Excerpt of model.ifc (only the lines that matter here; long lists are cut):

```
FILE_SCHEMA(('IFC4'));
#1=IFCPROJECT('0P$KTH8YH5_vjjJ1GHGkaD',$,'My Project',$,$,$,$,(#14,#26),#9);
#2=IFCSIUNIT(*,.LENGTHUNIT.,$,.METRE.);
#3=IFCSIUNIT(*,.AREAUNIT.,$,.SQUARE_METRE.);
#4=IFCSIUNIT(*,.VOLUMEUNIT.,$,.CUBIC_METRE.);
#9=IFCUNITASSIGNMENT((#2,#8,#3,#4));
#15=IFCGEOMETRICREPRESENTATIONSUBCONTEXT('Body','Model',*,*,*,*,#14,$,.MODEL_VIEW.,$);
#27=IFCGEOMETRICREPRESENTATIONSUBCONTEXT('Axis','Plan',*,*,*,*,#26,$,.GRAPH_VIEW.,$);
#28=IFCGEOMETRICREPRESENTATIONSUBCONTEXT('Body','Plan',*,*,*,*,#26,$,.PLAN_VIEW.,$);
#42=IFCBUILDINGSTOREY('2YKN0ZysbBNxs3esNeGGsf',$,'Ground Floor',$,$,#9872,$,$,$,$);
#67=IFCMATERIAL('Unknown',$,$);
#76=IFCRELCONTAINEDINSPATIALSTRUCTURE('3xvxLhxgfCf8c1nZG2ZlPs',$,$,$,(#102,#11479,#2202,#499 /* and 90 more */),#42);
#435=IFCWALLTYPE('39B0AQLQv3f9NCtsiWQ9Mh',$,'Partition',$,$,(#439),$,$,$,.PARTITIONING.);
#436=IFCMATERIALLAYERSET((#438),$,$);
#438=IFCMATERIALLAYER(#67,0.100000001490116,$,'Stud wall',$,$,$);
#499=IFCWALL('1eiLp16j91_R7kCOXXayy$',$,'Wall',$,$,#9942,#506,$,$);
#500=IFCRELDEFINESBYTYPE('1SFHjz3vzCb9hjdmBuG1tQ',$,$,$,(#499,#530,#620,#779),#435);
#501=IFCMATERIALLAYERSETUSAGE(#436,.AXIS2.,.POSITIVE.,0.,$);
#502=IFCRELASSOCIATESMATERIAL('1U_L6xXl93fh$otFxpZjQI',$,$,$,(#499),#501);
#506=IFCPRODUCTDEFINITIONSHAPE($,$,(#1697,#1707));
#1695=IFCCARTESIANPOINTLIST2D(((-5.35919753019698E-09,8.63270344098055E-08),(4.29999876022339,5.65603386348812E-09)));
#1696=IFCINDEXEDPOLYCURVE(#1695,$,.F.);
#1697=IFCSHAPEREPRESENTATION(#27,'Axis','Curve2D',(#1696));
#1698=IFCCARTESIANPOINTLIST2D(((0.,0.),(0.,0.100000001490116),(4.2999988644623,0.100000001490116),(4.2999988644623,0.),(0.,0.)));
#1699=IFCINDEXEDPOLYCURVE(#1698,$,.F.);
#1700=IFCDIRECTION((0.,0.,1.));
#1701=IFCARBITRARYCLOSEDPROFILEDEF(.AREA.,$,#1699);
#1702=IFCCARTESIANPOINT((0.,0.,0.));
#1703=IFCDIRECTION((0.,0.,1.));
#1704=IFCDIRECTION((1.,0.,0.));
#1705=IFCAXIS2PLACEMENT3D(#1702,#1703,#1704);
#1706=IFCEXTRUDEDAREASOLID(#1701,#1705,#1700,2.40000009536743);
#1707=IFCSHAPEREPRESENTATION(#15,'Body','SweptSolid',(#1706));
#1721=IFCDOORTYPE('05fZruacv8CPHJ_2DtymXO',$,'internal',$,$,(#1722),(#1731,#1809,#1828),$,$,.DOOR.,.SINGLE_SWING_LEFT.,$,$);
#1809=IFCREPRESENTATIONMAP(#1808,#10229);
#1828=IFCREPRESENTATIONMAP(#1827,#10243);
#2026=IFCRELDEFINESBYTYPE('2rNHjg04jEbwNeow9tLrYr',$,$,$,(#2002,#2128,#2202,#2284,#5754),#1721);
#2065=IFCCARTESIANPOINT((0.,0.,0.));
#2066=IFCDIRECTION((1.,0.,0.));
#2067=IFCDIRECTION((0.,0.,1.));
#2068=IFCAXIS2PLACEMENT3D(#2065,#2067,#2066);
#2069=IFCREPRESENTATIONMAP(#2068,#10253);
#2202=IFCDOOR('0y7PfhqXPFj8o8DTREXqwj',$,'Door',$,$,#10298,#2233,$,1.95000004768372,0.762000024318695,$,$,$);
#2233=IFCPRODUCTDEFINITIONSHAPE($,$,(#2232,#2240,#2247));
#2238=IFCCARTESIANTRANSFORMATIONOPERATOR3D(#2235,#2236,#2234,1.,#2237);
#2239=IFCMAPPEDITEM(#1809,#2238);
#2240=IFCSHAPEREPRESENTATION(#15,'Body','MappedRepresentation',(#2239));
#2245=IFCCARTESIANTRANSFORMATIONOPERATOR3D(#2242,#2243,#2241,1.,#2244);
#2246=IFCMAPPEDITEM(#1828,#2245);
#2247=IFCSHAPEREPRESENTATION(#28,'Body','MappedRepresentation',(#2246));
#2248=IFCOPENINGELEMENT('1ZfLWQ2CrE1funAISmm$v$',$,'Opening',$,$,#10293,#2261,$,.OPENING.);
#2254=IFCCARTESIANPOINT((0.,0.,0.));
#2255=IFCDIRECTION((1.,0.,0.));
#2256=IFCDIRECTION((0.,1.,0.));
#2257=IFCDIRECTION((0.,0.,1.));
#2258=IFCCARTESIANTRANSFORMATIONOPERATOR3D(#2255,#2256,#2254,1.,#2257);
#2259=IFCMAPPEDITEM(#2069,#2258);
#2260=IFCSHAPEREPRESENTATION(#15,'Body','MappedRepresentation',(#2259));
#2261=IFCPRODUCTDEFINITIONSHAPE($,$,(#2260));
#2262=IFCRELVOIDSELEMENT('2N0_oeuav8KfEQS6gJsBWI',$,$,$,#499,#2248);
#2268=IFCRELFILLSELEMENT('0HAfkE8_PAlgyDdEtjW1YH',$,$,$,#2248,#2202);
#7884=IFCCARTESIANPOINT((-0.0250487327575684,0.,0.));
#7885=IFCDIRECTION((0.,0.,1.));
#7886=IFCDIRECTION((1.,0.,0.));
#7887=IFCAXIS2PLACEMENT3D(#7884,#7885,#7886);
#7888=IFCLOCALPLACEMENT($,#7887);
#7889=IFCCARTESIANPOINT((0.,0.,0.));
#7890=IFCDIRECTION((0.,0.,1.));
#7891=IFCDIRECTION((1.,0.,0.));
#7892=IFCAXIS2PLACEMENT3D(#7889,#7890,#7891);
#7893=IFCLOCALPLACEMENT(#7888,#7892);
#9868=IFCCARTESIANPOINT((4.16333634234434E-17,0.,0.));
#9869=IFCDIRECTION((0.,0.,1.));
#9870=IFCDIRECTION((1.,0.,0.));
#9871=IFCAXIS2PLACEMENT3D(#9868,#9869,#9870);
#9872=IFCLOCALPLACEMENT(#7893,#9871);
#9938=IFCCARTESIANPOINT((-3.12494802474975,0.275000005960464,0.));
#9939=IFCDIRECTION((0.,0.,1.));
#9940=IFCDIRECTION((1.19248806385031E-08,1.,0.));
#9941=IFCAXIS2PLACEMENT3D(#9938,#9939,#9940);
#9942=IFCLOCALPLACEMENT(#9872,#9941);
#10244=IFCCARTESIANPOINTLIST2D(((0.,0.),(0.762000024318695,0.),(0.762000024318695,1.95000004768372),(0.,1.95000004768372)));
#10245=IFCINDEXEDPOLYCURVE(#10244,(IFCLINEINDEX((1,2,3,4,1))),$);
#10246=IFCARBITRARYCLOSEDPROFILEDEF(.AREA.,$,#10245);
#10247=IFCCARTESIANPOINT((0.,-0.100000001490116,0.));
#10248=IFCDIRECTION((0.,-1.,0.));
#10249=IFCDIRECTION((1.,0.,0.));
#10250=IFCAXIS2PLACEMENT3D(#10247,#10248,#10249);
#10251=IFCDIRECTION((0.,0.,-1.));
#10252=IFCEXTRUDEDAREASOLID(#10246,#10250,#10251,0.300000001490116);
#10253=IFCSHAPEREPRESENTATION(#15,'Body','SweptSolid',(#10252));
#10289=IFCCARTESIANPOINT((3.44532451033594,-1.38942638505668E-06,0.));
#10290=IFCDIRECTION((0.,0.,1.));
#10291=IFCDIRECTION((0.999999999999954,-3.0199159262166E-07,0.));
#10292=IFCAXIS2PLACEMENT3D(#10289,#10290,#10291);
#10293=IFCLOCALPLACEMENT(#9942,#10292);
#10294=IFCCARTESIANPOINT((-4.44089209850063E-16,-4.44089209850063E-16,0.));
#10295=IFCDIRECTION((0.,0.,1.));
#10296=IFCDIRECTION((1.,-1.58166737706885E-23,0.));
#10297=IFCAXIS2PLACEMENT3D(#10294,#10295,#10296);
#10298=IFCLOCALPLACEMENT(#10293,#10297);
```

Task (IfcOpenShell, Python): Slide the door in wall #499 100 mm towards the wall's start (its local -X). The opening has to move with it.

```python
import ifcopenshell
import ifcopenshell.api.geometry
import ifcopenshell.util.placement
import ifcopenshell.util.unit

model = ifcopenshell.open("model.ifc")
unit_scale = ifcopenshell.util.unit.calculate_unit_scale(model)

door = model.by_id(2202)
opening = door.FillsVoids[0].RelatingOpeningElement
wall = opening.VoidsElements[0].RelatingBuildingElement

wall_matrix = ifcopenshell.util.placement.get_local_placement(wall.ObjectPlacement)
shift = wall_matrix[:3, 0] * -0.1 / unit_scale
before = ifcopenshell.util.placement.get_local_placement(door.ObjectPlacement)[:3, 3].copy()

# The door is placed relative to its opening, so it follows when the opening moves.
matrix = ifcopenshell.util.placement.get_local_placement(opening.ObjectPlacement)
matrix[:3, 3] += shift
ifcopenshell.api.geometry.edit_object_placement(
    model, product=opening, matrix=matrix, is_si=False, should_transform_children=True
)

after = ifcopenshell.util.placement.get_local_placement(door.ObjectPlacement)[:3, 3]
print("door moved by", (after - before).round(3) + 0.0)

model.write("model_edited.ifc")
```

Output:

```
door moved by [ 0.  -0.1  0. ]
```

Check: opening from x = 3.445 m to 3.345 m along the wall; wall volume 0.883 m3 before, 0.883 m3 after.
